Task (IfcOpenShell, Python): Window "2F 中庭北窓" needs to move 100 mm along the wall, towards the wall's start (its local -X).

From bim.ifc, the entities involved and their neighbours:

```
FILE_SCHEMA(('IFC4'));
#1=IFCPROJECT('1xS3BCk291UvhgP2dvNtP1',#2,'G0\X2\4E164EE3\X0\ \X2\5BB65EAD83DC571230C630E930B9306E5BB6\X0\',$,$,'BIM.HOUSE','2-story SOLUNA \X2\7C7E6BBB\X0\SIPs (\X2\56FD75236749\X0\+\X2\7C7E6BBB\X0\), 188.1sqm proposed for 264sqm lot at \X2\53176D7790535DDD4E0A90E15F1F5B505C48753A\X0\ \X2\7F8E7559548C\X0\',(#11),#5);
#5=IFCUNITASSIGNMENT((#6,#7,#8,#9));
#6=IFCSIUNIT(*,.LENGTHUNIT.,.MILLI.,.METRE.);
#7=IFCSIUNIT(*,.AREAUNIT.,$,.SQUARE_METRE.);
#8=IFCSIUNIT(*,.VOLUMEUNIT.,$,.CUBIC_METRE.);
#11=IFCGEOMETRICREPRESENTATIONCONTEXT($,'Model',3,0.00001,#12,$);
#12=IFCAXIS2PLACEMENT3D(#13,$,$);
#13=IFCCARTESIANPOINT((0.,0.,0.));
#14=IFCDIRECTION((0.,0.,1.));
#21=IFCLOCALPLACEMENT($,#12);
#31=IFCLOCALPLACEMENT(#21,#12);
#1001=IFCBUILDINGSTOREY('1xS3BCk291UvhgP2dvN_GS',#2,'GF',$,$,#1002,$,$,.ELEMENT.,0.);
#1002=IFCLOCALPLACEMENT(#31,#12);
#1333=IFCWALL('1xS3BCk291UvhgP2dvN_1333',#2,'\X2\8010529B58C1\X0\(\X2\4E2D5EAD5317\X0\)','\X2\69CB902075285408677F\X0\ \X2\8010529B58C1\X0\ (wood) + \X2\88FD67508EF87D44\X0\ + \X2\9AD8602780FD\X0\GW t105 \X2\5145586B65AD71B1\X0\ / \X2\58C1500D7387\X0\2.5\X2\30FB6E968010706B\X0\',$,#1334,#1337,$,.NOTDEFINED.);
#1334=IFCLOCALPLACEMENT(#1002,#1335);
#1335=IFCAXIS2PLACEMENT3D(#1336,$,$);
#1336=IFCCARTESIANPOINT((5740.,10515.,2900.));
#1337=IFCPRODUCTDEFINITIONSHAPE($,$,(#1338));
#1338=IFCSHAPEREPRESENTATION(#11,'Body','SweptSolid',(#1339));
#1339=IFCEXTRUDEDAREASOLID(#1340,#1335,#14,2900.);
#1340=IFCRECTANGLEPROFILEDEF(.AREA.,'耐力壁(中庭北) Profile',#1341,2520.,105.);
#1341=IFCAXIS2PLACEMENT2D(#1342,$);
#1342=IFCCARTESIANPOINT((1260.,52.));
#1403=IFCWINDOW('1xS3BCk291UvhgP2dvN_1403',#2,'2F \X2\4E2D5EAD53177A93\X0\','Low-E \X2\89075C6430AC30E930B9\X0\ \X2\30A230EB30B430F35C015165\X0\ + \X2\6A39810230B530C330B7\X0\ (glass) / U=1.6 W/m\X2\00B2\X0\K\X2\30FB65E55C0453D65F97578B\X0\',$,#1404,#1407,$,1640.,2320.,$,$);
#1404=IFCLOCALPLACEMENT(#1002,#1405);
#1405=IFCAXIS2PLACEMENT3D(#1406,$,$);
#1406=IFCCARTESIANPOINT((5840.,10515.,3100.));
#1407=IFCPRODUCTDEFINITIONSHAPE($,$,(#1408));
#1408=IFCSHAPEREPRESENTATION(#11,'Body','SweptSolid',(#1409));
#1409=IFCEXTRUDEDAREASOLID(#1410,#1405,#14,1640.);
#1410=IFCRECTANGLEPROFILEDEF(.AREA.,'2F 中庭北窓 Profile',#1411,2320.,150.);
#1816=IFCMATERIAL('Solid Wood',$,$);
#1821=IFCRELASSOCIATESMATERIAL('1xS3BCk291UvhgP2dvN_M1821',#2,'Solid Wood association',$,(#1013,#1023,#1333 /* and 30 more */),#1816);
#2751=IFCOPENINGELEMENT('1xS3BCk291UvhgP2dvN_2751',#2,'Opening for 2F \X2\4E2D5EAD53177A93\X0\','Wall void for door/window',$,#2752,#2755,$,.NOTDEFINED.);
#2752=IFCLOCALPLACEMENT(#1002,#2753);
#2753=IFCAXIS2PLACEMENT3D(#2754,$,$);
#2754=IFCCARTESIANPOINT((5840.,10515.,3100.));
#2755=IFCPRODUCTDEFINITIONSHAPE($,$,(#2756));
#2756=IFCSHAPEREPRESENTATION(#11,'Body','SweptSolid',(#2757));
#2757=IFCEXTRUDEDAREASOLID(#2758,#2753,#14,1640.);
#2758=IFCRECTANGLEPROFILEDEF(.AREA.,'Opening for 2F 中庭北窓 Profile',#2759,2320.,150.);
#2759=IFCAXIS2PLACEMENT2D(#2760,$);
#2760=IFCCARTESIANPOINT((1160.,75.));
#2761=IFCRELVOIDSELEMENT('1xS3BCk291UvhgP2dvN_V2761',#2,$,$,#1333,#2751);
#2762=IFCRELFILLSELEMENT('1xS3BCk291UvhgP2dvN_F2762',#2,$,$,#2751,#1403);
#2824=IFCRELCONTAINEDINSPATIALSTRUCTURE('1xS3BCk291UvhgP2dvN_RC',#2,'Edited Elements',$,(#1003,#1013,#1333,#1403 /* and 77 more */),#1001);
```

```python
import ifcopenshell
import ifcopenshell.api.geometry
import ifcopenshell.util.placement
import ifcopenshell.util.unit

model = ifcopenshell.open("bim.ifc")
unit_scale = ifcopenshell.util.unit.calculate_unit_scale(model)

window = model.by_guid("1xS3BCk291UvhgP2dvN_1403")
opening = window.FillsVoids[0].RelatingOpeningElement
wall = opening.VoidsElements[0].RelatingBuildingElement

wall_matrix = ifcopenshell.util.placement.get_local_placement(wall.ObjectPlacement)
shift = wall_matrix[:3, 0] * -0.1 / unit_scale
before = ifcopenshell.util.placement.get_local_placement(window.ObjectPlacement)[:3, 3].copy()

# The window is not placed relative to its opening, so move both.
for product in (opening, window):
    matrix = ifcopenshell.util.placement.get_local_placement(product.ObjectPlacement)
    matrix[:3, 3] += shift
    ifcopenshell.api.geometry.edit_object_placement(model, product=product, matrix=matrix, is_si=False)

after = ifcopenshell.util.placement.get_local_placement(window.ObjectPlacement)[:3, 3]
print("window moved by", (after - before).round(3) + 0.0)

model.write("bim_edited.ifc")
```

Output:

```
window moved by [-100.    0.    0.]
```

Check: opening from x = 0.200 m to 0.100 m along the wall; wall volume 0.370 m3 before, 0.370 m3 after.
